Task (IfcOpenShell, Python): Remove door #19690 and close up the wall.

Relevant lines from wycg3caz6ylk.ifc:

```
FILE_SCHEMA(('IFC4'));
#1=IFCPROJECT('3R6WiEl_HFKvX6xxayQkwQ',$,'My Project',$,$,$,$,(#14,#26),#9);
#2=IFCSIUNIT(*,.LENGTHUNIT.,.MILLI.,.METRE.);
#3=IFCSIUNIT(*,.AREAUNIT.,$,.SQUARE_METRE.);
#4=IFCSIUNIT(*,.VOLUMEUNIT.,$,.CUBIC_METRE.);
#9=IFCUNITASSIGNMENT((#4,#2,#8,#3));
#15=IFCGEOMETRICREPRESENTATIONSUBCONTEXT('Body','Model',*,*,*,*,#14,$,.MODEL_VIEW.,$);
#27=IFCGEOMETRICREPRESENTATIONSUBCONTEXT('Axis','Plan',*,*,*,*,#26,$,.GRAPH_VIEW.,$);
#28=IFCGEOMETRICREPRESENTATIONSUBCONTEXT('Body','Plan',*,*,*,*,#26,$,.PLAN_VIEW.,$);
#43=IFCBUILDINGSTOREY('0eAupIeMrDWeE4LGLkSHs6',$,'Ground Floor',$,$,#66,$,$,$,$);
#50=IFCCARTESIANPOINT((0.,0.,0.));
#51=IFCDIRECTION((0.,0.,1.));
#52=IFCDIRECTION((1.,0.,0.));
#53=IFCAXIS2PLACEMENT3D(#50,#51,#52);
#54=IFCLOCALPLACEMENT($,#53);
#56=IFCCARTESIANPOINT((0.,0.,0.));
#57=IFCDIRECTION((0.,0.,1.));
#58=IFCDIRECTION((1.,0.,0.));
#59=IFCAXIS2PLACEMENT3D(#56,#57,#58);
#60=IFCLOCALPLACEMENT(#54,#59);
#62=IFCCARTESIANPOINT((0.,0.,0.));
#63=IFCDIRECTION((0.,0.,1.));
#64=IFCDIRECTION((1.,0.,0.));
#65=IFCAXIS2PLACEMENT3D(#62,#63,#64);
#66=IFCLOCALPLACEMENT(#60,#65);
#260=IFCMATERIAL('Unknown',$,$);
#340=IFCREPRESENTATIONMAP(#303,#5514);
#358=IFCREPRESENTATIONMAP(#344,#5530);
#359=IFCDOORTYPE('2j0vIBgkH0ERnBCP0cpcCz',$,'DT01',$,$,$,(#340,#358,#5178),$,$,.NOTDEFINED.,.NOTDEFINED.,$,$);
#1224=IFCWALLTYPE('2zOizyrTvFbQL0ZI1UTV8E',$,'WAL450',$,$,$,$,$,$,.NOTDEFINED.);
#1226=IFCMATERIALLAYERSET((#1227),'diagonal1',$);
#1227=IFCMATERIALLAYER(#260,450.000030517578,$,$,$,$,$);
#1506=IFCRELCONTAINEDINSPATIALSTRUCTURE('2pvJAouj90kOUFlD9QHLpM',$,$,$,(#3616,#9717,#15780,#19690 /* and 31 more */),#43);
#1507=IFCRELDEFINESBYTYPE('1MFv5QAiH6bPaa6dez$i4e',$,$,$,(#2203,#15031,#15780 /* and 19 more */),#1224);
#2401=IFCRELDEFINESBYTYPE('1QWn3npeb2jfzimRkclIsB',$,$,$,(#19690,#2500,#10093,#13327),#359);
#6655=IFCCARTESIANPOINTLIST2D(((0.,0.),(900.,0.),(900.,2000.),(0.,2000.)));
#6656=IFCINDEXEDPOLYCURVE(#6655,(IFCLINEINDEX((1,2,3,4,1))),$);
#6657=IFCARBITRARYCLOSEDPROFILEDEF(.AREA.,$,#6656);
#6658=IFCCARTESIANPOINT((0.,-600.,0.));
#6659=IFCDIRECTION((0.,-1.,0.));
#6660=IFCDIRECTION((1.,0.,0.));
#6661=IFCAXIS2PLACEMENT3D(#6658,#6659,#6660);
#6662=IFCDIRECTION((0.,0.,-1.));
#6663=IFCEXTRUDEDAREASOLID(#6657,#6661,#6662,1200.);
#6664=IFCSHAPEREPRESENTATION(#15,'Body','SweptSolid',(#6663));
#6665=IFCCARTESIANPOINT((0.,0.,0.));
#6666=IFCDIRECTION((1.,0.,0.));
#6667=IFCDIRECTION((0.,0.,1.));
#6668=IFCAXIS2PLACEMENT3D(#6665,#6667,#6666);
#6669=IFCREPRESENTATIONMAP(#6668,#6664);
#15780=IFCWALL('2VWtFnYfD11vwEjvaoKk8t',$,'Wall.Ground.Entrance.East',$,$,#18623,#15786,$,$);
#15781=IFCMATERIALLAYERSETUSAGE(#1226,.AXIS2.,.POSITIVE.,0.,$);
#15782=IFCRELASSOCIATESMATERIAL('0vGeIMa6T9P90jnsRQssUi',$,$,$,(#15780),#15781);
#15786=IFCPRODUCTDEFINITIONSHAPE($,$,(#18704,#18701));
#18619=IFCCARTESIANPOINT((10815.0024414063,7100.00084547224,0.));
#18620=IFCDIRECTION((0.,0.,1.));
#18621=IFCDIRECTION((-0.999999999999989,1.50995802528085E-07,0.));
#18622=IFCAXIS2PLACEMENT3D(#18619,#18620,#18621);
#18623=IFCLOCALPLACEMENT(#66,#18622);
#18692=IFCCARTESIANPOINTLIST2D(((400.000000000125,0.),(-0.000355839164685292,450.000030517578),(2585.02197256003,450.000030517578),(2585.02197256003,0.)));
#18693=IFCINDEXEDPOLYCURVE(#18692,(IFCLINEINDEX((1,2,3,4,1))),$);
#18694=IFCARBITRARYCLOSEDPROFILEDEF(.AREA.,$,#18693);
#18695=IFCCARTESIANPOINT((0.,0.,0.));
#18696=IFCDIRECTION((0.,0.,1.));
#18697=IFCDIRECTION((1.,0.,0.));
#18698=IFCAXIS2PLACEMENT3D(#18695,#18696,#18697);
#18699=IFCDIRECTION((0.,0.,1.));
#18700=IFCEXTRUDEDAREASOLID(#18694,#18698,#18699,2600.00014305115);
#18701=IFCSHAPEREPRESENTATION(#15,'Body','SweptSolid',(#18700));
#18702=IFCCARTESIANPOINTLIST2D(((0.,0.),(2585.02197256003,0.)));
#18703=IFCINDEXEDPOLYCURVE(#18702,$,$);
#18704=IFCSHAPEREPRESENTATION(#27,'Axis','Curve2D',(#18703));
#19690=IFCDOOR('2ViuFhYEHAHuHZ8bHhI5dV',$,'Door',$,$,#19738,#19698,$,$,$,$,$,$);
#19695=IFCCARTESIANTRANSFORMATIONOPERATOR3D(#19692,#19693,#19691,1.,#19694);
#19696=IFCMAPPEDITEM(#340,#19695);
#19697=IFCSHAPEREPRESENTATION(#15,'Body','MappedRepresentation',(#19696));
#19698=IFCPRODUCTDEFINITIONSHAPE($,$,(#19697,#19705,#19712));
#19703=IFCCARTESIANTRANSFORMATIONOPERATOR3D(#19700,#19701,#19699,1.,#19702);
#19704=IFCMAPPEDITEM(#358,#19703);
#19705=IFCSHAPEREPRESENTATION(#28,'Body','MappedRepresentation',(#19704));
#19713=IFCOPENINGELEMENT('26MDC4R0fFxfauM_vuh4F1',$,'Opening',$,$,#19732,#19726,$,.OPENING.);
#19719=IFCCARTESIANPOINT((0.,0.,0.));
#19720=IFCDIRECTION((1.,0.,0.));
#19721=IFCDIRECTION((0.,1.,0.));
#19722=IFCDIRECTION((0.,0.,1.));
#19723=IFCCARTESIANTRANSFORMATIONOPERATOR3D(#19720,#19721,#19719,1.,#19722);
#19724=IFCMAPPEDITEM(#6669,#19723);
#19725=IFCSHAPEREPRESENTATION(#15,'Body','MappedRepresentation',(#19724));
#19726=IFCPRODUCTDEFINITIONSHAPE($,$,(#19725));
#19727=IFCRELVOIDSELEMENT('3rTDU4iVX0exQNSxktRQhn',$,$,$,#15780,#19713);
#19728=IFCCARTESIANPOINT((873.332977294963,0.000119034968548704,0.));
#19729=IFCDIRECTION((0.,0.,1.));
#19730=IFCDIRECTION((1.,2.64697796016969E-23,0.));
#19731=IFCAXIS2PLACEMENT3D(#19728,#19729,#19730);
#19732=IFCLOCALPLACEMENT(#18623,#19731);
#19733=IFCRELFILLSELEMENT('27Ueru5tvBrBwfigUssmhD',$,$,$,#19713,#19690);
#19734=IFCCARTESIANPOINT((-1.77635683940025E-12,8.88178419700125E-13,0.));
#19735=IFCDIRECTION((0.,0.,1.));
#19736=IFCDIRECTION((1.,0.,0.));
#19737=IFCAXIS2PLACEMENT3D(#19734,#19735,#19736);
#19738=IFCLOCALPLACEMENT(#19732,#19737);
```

```python
import ifcopenshell
import ifcopenshell.api.feature
import ifcopenshell.api.root
import ifcopenshell.geom
import ifcopenshell.util.shape

model = ifcopenshell.open("wycg3caz6ylk.ifc")
settings = ifcopenshell.geom.settings()


def volume(element):
    """Net volume in cubic metres, openings subtracted."""
    shape = ifcopenshell.geom.create_shape(settings, element)
    return ifcopenshell.util.shape.get_volume(shape.geometry)


door = model.by_guid("2ViuFhYEHAHuHZ8bHhI5dV")
opening = door.FillsVoids[0].RelatingOpeningElement
wall = opening.VoidsElements[0].RelatingBuildingElement
before = volume(wall)

ifcopenshell.api.root.remove_product(model, product=door)
ifcopenshell.api.feature.remove_feature(model, feature=opening)

after = volume(wall)

print(f"wall volume {before:.3f} -> {after:.3f} m3")

model.write("wycg3caz6ylk_rev.ifc")
```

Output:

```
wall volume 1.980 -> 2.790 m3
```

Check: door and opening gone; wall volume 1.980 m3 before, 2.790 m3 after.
